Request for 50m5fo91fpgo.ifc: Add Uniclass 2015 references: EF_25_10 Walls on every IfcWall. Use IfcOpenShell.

First a look at what the model holds.

```python
import ifcopenshell

model = ifcopenshell.open("50m5fo91fpgo.ifc")
print(model.schema)
print("classifications:", [c.Name for c in model.by_type("IfcClassification")])
for ifc_class in ("IfcDoor", "IfcRoof", "IfcStair", "IfcWall", "IfcWindow"):
    print(ifc_class, len(model.by_type(ifc_class)))
```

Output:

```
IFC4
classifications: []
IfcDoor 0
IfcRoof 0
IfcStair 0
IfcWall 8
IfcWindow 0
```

```python
import ifcopenshell
import ifcopenshell.api.classification

model = ifcopenshell.open("50m5fo91fpgo.ifc")

system = ifcopenshell.api.classification.add_classification(model, classification="Uniclass 2015")

codes = {
    "IfcWall": ("EF_25_10", "Walls"),
}
for ifc_class, (code, name) in codes.items():
    products = model.by_type(ifc_class)
    ifcopenshell.api.classification.add_reference(
        model, products=products, classification=system, identification=code, name=name
    )
    print(code, len(products))

model.write("50m5fo91fpgo_updated.ifc")
```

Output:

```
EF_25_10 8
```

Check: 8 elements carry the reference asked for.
